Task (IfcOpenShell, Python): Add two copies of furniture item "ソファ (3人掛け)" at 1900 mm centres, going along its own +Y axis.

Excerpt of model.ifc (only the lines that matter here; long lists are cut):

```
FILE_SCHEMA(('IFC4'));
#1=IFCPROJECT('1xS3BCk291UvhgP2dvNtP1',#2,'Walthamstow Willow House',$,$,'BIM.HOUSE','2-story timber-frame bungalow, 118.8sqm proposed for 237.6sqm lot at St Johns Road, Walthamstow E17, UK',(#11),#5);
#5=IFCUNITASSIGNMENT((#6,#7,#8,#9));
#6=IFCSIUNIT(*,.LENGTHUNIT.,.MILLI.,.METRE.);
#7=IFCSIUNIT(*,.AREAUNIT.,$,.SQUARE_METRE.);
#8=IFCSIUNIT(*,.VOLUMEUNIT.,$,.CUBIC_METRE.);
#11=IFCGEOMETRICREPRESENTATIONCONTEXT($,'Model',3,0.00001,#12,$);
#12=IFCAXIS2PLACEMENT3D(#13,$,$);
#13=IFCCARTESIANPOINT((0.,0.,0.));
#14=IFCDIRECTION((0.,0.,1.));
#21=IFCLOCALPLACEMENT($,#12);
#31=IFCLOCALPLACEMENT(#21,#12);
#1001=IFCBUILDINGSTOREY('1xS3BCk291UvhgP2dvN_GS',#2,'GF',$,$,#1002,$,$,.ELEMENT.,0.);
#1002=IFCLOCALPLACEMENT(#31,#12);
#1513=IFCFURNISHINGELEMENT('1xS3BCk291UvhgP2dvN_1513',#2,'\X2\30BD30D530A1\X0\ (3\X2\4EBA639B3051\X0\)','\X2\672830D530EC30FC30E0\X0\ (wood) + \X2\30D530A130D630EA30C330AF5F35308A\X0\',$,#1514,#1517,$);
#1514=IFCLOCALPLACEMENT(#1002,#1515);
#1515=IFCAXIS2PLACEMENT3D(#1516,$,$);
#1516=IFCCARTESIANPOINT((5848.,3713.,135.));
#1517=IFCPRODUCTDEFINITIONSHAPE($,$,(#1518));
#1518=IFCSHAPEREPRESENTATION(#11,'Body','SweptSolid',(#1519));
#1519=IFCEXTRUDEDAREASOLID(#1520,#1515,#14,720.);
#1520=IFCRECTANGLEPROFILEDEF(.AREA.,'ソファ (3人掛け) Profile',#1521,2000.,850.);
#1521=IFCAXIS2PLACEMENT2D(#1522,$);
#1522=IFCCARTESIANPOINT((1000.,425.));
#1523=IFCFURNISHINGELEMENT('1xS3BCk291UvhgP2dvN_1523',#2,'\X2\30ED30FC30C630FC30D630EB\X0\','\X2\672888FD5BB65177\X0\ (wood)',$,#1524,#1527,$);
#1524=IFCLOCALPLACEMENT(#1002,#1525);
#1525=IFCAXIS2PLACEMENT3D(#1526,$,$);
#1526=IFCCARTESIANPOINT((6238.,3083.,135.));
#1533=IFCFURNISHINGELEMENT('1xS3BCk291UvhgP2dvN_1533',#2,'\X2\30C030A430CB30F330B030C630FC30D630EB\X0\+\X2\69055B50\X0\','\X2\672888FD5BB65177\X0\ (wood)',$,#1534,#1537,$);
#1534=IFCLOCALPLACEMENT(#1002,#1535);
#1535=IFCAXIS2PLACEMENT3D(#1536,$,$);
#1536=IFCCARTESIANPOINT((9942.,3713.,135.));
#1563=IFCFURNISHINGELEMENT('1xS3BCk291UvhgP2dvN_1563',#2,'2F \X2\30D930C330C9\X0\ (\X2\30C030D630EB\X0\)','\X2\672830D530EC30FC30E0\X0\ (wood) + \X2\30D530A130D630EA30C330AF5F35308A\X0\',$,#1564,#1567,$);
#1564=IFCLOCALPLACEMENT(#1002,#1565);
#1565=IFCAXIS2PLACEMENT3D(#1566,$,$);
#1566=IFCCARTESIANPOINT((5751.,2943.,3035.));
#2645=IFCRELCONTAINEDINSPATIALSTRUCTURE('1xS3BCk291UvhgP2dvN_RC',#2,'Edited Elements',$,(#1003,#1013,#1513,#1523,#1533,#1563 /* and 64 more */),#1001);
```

```python
import ifcopenshell
import ifcopenshell.api.geometry
import ifcopenshell.api.root
import ifcopenshell.util.element
import ifcopenshell.util.placement
import ifcopenshell.util.unit

model = ifcopenshell.open("model.ifc")
unit_scale = ifcopenshell.util.unit.calculate_unit_scale(model)


def reuse_history(source, copy):
    """copy_class also copies each property set's owner history, people and application; keep the originals."""
    for rel in copy.IsDefinedBy:
        if rel.is_a("IfcRelDefinesByProperties") and (history := rel.RelatingPropertyDefinition.OwnerHistory):
            rel.RelatingPropertyDefinition.OwnerHistory = source.OwnerHistory
            ifcopenshell.util.element.remove_deep2(model, history)


source = model.by_guid("1xS3BCk291UvhgP2dvN_1513")
base = ifcopenshell.util.placement.get_local_placement(source.ObjectPlacement)
step = base[:3, 1] * 1.9 / unit_scale

for i in range(1, 3):
    copy = ifcopenshell.api.root.copy_class(model, product=source)
    copy.Representation = ifcopenshell.util.element.copy_deep(
        model, source.Representation, exclude=["IfcGeometricRepresentationContext", "IfcRepresentationMap"]
    )
    reuse_history(source, copy)
    matrix = base.copy()
    matrix[:3, 3] += i * step
    print("added at", matrix[:3, 3].round(3) + 0.0)
    ifcopenshell.api.geometry.edit_object_placement(model, product=copy, matrix=matrix, is_si=False)

model.write("model_updated.ifc")
```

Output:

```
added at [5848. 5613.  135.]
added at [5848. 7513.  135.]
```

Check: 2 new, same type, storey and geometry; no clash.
